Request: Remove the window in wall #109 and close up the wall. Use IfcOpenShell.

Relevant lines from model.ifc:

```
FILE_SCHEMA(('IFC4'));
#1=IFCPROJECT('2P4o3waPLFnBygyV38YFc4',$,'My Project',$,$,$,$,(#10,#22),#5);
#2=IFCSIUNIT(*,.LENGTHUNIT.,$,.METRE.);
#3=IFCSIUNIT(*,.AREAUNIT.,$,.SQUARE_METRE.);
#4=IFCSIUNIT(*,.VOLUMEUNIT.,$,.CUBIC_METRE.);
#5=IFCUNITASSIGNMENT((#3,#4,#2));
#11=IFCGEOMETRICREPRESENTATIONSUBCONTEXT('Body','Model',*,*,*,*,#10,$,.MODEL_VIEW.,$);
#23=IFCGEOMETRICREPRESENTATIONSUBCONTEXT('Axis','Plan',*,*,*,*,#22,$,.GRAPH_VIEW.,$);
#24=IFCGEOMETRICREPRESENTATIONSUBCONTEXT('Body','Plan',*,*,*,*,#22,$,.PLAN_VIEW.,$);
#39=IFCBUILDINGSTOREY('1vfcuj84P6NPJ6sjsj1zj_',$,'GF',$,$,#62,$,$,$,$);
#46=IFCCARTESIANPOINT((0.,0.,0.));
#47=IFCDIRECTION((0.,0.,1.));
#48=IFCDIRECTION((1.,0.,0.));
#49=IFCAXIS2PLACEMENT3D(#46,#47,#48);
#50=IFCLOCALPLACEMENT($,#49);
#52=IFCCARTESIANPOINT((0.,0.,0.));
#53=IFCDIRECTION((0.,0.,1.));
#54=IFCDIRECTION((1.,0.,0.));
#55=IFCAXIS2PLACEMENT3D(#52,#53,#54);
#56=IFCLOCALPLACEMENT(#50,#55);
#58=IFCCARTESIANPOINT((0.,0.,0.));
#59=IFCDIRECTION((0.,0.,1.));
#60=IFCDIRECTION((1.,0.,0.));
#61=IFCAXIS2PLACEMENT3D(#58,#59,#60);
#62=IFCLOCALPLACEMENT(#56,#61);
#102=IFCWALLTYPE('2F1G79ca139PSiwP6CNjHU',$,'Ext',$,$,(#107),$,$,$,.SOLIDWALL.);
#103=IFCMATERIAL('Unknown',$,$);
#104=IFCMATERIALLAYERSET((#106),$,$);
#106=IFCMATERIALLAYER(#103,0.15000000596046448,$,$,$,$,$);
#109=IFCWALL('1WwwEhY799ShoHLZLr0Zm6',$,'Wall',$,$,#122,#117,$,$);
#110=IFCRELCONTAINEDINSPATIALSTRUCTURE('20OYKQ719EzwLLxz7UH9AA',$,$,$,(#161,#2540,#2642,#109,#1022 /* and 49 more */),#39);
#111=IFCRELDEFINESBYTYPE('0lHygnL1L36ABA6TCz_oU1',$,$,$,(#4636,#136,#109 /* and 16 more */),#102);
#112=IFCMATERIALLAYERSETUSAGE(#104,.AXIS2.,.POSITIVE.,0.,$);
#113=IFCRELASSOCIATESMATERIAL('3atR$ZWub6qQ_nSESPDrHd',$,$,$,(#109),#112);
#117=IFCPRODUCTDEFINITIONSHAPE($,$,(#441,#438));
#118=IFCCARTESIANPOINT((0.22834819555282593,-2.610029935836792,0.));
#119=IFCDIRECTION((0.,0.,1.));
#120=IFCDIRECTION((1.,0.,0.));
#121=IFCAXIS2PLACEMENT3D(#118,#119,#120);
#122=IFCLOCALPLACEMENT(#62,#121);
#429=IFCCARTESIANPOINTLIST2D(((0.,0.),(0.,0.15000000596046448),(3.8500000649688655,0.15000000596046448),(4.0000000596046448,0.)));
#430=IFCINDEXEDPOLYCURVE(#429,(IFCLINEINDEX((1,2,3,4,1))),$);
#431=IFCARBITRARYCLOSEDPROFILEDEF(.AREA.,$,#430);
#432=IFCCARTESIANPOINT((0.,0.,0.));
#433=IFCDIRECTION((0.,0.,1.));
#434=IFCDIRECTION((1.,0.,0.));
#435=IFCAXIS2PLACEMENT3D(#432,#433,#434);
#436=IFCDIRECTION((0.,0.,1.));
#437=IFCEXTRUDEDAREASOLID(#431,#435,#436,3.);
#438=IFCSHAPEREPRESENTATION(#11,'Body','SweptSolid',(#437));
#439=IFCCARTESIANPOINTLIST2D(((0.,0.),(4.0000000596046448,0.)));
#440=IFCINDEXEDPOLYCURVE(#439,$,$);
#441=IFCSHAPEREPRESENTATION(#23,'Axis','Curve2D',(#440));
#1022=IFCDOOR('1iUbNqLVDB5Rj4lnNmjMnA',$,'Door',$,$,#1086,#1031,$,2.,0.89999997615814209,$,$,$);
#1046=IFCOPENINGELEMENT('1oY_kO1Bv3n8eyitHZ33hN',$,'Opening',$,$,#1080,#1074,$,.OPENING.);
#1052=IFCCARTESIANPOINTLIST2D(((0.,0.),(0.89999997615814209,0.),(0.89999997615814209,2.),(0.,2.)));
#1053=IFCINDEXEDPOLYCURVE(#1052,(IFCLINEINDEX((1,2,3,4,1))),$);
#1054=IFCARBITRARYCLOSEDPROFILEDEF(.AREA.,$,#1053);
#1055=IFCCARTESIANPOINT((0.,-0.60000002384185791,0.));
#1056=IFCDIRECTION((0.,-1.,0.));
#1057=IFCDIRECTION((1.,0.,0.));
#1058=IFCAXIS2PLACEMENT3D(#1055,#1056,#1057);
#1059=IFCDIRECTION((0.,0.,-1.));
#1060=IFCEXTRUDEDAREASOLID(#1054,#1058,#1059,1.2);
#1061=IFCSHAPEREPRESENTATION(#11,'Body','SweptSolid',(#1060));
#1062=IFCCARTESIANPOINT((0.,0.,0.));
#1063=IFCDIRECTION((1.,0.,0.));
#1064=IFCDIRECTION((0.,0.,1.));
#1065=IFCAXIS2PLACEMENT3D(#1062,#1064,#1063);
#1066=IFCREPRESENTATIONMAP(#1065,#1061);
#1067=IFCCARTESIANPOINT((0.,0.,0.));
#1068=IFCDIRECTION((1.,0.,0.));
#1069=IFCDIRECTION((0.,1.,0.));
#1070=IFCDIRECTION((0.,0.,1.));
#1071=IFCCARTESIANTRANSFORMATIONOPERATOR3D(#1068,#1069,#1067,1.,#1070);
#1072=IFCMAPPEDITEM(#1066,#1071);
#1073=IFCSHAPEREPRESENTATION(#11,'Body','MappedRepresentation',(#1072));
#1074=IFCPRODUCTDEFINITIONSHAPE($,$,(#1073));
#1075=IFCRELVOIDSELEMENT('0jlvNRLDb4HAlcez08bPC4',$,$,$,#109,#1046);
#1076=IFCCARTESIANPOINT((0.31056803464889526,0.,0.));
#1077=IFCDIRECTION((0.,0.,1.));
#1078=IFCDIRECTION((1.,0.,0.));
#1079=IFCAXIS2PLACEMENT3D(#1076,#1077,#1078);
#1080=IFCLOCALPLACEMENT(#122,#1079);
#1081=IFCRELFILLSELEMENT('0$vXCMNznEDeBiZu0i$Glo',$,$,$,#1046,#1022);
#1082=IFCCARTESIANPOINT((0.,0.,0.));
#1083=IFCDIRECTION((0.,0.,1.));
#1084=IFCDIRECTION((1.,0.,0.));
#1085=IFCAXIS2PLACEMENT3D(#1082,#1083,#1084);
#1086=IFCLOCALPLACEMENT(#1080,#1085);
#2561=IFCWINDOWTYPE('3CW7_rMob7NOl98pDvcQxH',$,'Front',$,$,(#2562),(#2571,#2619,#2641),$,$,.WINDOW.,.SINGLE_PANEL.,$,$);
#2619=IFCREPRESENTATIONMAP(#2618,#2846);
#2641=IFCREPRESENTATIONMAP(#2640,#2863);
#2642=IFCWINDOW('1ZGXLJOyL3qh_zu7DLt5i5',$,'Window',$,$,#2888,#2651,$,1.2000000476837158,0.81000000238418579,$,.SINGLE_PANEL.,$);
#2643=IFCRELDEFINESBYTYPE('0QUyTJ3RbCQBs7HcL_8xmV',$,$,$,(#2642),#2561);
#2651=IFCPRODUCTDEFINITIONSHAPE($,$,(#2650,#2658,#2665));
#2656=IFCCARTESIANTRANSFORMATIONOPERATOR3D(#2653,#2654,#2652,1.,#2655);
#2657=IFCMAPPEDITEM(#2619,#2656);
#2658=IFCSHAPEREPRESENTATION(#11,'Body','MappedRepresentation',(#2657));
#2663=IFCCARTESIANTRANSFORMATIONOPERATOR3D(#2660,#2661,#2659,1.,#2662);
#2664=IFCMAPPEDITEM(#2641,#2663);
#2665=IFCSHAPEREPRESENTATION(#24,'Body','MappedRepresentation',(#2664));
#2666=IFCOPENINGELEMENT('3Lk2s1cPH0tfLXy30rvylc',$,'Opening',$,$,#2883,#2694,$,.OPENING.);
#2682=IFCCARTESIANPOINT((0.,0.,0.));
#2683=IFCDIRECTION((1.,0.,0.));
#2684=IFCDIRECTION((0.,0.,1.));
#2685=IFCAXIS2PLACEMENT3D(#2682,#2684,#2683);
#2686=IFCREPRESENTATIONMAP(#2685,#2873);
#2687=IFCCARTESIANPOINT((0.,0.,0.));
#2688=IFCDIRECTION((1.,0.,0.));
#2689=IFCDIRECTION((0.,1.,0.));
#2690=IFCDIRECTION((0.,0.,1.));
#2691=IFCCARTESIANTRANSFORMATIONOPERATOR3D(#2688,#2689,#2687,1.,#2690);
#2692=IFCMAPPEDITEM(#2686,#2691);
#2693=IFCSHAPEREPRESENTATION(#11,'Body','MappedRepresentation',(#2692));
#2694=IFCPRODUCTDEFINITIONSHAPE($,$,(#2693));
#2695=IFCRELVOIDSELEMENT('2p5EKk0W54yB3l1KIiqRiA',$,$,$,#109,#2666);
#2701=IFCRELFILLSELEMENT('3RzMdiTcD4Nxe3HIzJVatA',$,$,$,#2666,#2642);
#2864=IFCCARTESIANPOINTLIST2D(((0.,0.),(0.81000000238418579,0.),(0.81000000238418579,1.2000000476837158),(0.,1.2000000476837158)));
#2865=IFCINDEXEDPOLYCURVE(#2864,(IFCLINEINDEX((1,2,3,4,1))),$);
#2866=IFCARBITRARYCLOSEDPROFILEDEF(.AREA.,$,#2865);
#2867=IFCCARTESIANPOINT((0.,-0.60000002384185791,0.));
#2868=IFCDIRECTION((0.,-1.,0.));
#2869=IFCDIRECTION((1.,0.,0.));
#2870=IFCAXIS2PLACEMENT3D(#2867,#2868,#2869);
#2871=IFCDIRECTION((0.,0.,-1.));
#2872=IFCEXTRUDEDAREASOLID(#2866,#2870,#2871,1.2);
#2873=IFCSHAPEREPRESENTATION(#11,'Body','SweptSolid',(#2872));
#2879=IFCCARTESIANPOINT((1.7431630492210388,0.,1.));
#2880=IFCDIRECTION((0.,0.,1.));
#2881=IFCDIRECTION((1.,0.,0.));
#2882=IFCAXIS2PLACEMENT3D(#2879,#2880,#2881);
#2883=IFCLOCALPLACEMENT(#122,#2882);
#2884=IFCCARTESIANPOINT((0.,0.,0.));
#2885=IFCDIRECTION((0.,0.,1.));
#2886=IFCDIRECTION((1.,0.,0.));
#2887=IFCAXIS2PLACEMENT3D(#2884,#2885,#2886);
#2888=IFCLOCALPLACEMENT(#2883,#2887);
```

```python
import ifcopenshell
import ifcopenshell.api.feature
import ifcopenshell.api.root
import ifcopenshell.geom
import ifcopenshell.util.shape

model = ifcopenshell.open("model.ifc")
settings = ifcopenshell.geom.settings()


def volume(element):
    """Net volume in cubic metres, openings subtracted."""
    shape = ifcopenshell.geom.create_shape(settings, element)
    return ifcopenshell.util.shape.get_volume(shape.geometry)


window = model.by_id(2642)
opening = window.FillsVoids[0].RelatingOpeningElement
wall = opening.VoidsElements[0].RelatingBuildingElement
before = volume(wall)

ifcopenshell.api.root.remove_product(model, product=window)
ifcopenshell.api.feature.remove_feature(model, feature=opening)

after = volume(wall)

print(f"wall volume {before:.3f} -> {after:.3f} m3")

model.write("model_updated.ifc")
```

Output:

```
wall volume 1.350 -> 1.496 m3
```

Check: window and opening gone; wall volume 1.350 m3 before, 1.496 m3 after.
